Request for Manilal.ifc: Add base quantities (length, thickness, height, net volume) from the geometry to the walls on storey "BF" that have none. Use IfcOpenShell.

First a look at what the model holds.

```python
import ifcopenshell
import ifcopenshell.util.element
import ifcopenshell.util.unit

model = ifcopenshell.open("Manilal.ifc")
print(model.schema)
for unit_type in ("LENGTHUNIT", "AREAUNIT", "VOLUMEUNIT"):
    print(unit_type, ifcopenshell.util.unit.calculate_unit_scale(model, unit_type))
storey = next(s for s in model.by_type("IfcBuildingStorey") if s.Name == "BF")
walls = [e for e in ifcopenshell.util.element.get_decomposition(storey) if e.is_a("IfcWall")]
for e in sorted(walls, key=lambda e: e.id()):
    print(e.id(), e.is_a(), e.Name, list(ifcopenshell.util.element.get_psets(e, qtos_only=True)), sep=" | ")
```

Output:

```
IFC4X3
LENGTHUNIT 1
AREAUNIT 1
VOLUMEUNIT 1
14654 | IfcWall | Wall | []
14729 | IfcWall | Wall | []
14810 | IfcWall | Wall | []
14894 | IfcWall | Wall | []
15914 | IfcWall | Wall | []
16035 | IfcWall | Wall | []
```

```python
import ifcopenshell
import ifcopenshell.api.pset
import ifcopenshell.geom
import ifcopenshell.util.element
import ifcopenshell.util.shape
import ifcopenshell.util.unit

model = ifcopenshell.open("Manilal.ifc")
unit_scale = ifcopenshell.util.unit.calculate_unit_scale(model)
volume_scale = ifcopenshell.util.unit.calculate_unit_scale(model, "VOLUMEUNIT")
settings = ifcopenshell.geom.settings()

storey = next(s for s in model.by_type("IfcBuildingStorey") if s.Name == "BF")
walls = [e for e in ifcopenshell.util.element.get_decomposition(storey) if e.is_a("IfcWall")]

for e in sorted(walls, key=lambda e: e.id()):
    if ifcopenshell.util.element.get_psets(e, qtos_only=True, should_inherit=False):
        continue
    # Geometry comes back in metres, in the element's own axes.
    shape = ifcopenshell.geom.create_shape(settings, e)
    values = {
        "Length": ifcopenshell.util.shape.get_x(shape.geometry) / unit_scale,
        "Width": ifcopenshell.util.shape.get_y(shape.geometry) / unit_scale,
        "Height": ifcopenshell.util.shape.get_z(shape.geometry) / unit_scale,
        "NetVolume": ifcopenshell.util.shape.get_volume(shape.geometry) / volume_scale,
    }
    qto = ifcopenshell.api.pset.add_qto(model, product=e, name="Qto_WallBaseQuantities")
    ifcopenshell.api.pset.edit_qto(model, qto=qto, properties=values)
    print(e.id(), {k: round(v, 3) for k, v in values.items()})

model.write("Manilal_updated.ifc")
```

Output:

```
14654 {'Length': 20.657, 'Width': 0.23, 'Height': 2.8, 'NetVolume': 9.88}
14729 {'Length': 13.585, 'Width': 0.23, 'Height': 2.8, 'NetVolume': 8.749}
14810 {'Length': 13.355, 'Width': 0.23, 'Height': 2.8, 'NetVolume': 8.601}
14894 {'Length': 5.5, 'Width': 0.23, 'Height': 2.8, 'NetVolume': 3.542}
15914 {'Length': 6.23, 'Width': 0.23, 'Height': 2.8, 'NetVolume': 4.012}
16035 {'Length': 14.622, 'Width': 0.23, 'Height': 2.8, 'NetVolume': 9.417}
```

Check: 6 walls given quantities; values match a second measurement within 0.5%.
